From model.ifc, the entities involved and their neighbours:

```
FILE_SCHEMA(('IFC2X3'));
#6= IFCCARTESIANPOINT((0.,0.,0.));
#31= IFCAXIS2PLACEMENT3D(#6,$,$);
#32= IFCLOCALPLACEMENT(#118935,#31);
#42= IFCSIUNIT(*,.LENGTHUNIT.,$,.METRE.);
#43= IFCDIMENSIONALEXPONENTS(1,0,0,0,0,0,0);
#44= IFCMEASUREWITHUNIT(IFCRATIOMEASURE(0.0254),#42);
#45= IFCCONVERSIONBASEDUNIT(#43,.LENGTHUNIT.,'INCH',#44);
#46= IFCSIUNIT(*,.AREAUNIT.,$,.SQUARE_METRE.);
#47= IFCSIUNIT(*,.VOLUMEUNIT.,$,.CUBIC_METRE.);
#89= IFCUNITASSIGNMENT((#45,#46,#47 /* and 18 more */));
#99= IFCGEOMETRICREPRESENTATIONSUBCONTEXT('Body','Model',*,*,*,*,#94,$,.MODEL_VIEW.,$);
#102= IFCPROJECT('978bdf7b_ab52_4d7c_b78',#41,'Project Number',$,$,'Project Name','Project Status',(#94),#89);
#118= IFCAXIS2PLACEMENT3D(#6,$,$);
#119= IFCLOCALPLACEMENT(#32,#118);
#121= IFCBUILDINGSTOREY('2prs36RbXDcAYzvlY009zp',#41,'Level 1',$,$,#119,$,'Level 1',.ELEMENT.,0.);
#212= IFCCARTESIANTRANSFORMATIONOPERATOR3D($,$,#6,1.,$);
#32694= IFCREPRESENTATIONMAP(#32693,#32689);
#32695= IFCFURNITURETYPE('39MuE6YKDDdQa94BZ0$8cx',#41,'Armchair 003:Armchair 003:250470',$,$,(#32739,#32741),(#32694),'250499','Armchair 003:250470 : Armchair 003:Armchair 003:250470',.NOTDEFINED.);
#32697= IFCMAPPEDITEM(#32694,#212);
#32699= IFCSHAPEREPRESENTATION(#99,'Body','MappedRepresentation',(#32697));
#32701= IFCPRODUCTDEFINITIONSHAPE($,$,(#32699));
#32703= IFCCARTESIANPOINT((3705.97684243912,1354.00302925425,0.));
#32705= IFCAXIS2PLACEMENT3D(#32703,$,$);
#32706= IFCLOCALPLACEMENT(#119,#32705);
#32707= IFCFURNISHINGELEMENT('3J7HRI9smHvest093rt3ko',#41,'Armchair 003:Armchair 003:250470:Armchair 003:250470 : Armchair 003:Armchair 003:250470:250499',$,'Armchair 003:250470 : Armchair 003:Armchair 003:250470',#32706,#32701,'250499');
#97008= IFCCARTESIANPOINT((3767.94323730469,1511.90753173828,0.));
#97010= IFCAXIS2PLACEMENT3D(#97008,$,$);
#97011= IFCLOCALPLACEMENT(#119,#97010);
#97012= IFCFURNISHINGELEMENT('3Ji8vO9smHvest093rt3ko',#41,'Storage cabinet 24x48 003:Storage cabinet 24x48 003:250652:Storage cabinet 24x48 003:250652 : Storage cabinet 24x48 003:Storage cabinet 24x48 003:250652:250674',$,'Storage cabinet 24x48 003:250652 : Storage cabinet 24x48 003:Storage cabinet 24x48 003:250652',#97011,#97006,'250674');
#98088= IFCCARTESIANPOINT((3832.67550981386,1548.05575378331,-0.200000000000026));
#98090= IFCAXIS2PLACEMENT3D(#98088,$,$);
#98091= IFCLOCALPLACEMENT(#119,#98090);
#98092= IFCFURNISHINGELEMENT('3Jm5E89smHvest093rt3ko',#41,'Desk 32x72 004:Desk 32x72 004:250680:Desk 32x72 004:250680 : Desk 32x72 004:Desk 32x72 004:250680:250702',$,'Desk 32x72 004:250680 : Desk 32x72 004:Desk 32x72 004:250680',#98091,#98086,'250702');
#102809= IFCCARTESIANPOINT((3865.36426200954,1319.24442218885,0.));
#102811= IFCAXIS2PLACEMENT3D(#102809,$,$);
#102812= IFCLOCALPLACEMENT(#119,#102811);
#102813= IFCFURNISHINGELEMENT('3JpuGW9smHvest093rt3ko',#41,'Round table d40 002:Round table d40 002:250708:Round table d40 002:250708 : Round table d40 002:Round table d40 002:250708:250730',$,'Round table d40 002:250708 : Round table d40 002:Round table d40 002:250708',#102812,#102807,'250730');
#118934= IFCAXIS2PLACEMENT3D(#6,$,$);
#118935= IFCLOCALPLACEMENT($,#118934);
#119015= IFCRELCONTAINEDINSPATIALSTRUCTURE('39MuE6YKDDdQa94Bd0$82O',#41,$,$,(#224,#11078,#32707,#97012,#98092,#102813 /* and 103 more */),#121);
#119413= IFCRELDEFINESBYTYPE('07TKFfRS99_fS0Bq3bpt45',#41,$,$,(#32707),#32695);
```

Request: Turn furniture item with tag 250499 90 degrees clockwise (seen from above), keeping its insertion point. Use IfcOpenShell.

```python
import ifcopenshell
import ifcopenshell.api.geometry
import ifcopenshell.util.placement

model = ifcopenshell.open("model.ifc")

item = model.by_guid("3J7HRI9smHvest093rt3ko")
matrix = ifcopenshell.util.placement.get_local_placement(item.ObjectPlacement)
matrix = matrix @ ifcopenshell.util.placement.rotation(-90, "Z")
ifcopenshell.api.geometry.edit_object_placement(model, product=item, matrix=matrix, is_si=False)

print(ifcopenshell.util.placement.get_local_placement(item.ObjectPlacement).round(3) + 0.0)

model.write("model-out.ifc")
```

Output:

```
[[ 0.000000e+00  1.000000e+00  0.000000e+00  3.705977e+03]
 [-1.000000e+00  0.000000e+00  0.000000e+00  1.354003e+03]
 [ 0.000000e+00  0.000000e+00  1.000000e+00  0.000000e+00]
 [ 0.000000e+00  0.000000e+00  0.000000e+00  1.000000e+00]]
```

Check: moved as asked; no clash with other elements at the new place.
